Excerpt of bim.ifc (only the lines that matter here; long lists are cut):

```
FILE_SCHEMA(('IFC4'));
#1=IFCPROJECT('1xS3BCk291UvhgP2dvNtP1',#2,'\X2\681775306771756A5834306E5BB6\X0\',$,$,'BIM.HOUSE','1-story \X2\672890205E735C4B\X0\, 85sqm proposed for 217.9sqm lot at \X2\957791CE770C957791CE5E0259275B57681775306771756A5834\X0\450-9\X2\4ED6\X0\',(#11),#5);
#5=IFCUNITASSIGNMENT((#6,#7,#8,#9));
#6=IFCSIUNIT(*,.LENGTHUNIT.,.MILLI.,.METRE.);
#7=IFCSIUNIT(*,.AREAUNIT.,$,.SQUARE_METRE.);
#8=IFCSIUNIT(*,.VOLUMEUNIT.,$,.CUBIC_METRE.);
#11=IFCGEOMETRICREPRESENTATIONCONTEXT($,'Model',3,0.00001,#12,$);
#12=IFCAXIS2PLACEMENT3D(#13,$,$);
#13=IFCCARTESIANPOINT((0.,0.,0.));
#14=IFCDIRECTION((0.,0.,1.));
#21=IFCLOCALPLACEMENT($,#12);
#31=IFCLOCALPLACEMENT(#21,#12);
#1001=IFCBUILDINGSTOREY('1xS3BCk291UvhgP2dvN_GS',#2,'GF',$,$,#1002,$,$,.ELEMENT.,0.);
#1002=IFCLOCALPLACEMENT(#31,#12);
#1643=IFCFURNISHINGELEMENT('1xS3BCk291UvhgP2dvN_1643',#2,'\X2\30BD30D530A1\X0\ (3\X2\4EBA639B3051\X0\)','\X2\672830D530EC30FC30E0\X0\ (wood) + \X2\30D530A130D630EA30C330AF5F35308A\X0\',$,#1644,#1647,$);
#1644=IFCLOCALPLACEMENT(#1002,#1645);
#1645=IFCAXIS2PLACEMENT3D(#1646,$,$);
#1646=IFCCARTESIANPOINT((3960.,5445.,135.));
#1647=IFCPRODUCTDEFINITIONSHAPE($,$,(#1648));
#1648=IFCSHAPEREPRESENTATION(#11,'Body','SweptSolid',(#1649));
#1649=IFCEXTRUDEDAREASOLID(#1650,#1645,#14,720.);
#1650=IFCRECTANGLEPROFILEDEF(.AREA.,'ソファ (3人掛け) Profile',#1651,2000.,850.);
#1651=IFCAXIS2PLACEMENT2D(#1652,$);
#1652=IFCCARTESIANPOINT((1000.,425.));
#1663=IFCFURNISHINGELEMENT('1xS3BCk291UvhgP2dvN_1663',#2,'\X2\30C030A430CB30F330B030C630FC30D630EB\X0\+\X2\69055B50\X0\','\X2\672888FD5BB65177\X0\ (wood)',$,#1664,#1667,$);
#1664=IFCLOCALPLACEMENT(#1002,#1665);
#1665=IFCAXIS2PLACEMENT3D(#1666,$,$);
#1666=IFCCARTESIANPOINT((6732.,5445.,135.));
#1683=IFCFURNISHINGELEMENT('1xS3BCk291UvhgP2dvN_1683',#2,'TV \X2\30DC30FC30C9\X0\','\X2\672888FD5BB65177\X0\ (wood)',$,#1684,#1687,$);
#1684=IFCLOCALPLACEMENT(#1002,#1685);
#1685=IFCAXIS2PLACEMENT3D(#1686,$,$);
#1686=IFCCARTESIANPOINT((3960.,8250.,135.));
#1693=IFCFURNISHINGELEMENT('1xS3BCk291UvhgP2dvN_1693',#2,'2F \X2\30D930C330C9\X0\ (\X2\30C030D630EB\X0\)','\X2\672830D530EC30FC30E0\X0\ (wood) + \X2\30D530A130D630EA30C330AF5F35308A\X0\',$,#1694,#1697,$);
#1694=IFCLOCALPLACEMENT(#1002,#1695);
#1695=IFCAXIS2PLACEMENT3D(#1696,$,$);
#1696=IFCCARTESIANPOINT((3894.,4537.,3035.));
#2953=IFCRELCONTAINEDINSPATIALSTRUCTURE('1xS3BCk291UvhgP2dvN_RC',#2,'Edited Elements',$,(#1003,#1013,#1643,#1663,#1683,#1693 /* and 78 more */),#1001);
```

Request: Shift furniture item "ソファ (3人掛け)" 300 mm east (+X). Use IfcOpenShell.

```python
import ifcopenshell
import ifcopenshell.api.geometry
import ifcopenshell.util.placement

model = ifcopenshell.open("bim.ifc")

item = model.by_id(1643)
matrix = ifcopenshell.util.placement.get_local_placement(item.ObjectPlacement)
matrix[0, 3] += 300.0
ifcopenshell.api.geometry.edit_object_placement(model, product=item, matrix=matrix, is_si=False)

print(ifcopenshell.util.placement.get_local_placement(item.ObjectPlacement).round(3) + 0.0)

model.write("bim-out.ifc")
```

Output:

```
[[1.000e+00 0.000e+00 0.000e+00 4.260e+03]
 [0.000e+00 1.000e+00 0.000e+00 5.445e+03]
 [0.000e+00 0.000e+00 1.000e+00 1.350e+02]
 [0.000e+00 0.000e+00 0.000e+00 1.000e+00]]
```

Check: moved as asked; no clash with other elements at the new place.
